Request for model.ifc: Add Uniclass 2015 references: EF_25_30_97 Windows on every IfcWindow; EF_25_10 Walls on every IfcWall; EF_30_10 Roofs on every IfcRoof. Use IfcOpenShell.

First a look at what the model holds.

```python
import ifcopenshell

model = ifcopenshell.open("model.ifc")
print(model.schema)
print("classifications:", [c.Name for c in model.by_type("IfcClassification")])
for ifc_class in ("IfcDoor", "IfcRoof", "IfcStair", "IfcWall", "IfcWindow"):
    print(ifc_class, len(model.by_type(ifc_class)))
```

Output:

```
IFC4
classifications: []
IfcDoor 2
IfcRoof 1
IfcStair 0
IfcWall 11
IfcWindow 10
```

```python
import ifcopenshell
import ifcopenshell.api.classification

model = ifcopenshell.open("model.ifc")

system = ifcopenshell.api.classification.add_classification(model, classification="Uniclass 2015")

codes = {
    "IfcWindow": ("EF_25_30_97", "Windows"),
    "IfcWall": ("EF_25_10", "Walls"),
    "IfcRoof": ("EF_30_10", "Roofs"),
}
for ifc_class, (code, name) in codes.items():
    products = model.by_type(ifc_class)
    ifcopenshell.api.classification.add_reference(
        model, products=products, classification=system, identification=code, name=name
    )
    print(code, len(products))

model.write("model_edited.ifc")
```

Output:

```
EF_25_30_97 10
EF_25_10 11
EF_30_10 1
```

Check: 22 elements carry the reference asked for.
